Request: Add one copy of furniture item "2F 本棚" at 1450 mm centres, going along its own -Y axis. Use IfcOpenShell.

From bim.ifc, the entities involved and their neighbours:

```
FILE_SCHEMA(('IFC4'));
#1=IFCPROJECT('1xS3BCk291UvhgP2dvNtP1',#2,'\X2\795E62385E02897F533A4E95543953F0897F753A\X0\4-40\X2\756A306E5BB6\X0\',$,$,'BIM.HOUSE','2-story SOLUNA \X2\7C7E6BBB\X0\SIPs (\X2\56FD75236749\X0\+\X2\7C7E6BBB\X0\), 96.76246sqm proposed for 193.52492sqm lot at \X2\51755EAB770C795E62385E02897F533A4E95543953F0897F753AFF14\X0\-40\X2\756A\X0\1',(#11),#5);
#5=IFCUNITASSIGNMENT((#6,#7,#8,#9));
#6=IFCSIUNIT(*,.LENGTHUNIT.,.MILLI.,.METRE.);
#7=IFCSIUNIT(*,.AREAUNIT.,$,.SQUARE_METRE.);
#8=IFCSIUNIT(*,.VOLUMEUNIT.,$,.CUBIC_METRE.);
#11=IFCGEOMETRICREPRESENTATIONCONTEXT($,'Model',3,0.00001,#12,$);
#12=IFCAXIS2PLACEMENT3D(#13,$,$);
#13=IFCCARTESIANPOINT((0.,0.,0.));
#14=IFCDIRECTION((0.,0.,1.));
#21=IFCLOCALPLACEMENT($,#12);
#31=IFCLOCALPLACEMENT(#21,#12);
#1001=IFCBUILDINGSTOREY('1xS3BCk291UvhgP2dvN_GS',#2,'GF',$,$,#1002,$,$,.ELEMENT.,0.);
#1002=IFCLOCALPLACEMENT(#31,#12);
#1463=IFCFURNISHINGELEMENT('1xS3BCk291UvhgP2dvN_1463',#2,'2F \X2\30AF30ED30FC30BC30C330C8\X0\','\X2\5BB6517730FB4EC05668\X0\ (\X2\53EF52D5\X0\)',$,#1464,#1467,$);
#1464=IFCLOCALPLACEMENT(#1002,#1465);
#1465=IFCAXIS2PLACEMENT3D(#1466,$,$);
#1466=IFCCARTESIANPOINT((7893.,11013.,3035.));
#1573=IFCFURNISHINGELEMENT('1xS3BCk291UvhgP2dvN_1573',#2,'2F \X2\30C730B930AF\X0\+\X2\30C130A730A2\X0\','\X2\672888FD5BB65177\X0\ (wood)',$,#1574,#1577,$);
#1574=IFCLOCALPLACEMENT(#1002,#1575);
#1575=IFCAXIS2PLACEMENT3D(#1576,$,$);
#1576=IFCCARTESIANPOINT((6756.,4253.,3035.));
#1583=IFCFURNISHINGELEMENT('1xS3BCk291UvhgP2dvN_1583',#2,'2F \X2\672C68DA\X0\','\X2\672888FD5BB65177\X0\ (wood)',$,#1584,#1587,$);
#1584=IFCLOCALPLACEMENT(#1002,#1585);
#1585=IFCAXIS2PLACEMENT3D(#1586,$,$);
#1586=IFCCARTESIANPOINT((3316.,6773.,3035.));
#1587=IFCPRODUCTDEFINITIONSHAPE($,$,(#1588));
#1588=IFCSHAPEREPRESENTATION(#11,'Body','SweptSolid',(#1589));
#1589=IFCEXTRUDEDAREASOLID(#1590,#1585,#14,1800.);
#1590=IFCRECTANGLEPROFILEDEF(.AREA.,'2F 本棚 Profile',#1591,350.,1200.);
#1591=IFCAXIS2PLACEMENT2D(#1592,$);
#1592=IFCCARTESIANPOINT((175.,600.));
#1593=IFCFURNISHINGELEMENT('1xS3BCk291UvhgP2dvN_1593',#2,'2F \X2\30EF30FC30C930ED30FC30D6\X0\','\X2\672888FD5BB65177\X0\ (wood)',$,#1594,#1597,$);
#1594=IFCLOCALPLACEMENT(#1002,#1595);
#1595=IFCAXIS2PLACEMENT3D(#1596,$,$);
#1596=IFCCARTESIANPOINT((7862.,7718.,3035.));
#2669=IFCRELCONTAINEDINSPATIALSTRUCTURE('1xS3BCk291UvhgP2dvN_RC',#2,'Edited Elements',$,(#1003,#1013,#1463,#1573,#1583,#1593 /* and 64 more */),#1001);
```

```python
import ifcopenshell
import ifcopenshell.api.geometry
import ifcopenshell.api.root
import ifcopenshell.util.element
import ifcopenshell.util.placement

model = ifcopenshell.open("bim.ifc")


def reuse_history(source, copy):
    """copy_class also copies each property set's owner history, people and application; keep the originals."""
    for rel in copy.IsDefinedBy:
        if rel.is_a("IfcRelDefinesByProperties") and (history := rel.RelatingPropertyDefinition.OwnerHistory):
            rel.RelatingPropertyDefinition.OwnerHistory = source.OwnerHistory
            ifcopenshell.util.element.remove_deep2(model, history)


source = model.by_id(1583)
base = ifcopenshell.util.placement.get_local_placement(source.ObjectPlacement)
step = -base[:3, 1] * 1450.0

for i in range(1, 2):
    copy = ifcopenshell.api.root.copy_class(model, product=source)
    copy.Representation = ifcopenshell.util.element.copy_deep(
        model, source.Representation, exclude=["IfcGeometricRepresentationContext", "IfcRepresentationMap"]
    )
    reuse_history(source, copy)
    matrix = base.copy()
    matrix[:3, 3] += i * step
    print("added at", matrix[:3, 3].round(3) + 0.0)
    ifcopenshell.api.geometry.edit_object_placement(model, product=copy, matrix=matrix, is_si=False)

model.write("bim_v2.ifc")
```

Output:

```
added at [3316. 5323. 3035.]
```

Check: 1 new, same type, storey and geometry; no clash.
